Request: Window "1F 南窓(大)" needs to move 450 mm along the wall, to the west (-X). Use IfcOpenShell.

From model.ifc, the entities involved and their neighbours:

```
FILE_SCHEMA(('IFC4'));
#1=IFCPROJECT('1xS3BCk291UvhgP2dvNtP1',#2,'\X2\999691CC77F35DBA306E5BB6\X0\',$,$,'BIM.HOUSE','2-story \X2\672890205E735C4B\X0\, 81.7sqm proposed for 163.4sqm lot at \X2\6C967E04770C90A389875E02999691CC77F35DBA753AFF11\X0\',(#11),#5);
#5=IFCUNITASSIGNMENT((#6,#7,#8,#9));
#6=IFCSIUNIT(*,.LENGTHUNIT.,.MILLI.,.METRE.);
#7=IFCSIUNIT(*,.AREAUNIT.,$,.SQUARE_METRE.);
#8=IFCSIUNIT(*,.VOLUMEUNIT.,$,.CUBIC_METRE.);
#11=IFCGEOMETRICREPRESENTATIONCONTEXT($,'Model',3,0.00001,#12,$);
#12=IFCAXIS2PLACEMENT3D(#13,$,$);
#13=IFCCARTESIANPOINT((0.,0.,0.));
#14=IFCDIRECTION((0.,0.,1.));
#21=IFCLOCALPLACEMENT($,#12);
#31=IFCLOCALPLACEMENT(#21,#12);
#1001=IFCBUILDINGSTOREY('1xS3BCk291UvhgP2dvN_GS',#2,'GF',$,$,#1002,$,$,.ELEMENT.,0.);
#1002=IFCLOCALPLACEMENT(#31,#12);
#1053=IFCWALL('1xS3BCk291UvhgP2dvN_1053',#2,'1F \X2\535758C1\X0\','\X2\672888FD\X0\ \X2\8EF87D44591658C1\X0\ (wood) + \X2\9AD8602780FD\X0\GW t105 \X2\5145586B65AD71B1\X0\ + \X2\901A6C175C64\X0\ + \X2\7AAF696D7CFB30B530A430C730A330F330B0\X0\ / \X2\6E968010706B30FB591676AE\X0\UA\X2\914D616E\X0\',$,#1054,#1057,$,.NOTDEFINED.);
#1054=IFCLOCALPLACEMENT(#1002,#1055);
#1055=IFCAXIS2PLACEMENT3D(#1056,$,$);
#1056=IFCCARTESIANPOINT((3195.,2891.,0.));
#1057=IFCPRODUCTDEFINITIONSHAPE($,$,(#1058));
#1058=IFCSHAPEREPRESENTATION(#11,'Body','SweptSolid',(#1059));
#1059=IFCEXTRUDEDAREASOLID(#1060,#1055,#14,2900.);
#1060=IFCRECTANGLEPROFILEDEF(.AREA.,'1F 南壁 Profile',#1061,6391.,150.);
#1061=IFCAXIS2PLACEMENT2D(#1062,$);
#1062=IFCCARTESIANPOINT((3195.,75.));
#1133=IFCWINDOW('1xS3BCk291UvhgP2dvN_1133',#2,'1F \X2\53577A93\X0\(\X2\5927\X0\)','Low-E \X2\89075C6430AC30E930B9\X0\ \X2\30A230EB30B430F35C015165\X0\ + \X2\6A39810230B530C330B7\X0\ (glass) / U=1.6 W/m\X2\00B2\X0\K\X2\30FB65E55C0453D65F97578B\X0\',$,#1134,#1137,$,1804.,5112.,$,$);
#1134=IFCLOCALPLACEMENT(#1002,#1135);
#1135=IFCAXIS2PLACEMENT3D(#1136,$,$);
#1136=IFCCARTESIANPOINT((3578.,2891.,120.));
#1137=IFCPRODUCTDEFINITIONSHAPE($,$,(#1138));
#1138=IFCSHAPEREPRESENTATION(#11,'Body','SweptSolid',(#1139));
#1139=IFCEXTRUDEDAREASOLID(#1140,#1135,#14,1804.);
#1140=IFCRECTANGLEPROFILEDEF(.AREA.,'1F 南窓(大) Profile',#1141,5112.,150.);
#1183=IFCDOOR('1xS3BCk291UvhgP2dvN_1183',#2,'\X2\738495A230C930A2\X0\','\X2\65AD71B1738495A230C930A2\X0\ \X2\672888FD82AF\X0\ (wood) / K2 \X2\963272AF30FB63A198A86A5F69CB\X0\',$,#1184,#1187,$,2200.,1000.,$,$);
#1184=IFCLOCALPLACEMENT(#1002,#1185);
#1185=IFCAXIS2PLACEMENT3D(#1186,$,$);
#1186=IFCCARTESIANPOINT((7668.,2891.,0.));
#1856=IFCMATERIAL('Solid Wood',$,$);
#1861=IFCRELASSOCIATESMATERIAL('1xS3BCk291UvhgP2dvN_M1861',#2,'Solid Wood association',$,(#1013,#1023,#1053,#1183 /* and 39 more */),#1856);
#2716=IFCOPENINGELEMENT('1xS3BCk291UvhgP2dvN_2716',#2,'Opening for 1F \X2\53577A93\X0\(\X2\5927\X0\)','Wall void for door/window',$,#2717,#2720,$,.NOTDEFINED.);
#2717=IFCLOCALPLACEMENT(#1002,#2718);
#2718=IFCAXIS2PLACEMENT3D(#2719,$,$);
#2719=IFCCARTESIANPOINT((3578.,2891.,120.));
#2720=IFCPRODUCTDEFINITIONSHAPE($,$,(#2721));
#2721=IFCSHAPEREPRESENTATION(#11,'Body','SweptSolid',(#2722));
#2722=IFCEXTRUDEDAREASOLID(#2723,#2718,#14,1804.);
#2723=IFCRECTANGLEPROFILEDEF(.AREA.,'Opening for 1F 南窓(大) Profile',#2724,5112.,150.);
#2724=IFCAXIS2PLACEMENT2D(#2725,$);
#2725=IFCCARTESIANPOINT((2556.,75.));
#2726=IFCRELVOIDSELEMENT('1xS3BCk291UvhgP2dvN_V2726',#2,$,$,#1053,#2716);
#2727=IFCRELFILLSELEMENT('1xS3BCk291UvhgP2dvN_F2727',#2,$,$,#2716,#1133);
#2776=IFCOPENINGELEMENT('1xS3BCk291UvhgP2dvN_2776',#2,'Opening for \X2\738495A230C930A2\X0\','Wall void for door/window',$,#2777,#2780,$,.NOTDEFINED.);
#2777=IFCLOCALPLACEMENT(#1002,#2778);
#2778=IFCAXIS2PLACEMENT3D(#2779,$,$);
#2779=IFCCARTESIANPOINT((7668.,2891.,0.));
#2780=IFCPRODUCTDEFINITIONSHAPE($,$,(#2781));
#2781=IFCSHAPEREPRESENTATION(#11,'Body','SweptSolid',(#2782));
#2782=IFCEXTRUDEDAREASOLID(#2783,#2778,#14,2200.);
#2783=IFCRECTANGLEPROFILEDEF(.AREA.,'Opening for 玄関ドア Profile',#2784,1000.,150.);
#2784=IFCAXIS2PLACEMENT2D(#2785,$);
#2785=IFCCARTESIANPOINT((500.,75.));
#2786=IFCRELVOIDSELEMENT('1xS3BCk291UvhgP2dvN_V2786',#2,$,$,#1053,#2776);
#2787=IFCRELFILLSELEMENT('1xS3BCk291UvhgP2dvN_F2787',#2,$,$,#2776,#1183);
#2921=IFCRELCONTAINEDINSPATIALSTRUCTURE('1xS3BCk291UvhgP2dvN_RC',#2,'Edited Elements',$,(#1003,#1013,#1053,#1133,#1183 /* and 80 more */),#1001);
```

```python
import ifcopenshell
import ifcopenshell.api.geometry
import ifcopenshell.util.placement

model = ifcopenshell.open("model.ifc")

window = model.by_id(1133)
opening = window.FillsVoids[0].RelatingOpeningElement
wall = opening.VoidsElements[0].RelatingBuildingElement

wall_matrix = ifcopenshell.util.placement.get_local_placement(wall.ObjectPlacement)
shift = wall_matrix[:3, 0] * -450.0
before = ifcopenshell.util.placement.get_local_placement(window.ObjectPlacement)[:3, 3].copy()

# The window is not placed relative to its opening, so move both.
for product in (opening, window):
    matrix = ifcopenshell.util.placement.get_local_placement(product.ObjectPlacement)
    matrix[:3, 3] += shift
    ifcopenshell.api.geometry.edit_object_placement(model, product=product, matrix=matrix, is_si=False)

after = ifcopenshell.util.placement.get_local_placement(window.ObjectPlacement)[:3, 3]
print("window moved by", (after - before).round(3) + 0.0)

model.write("model_v2.ifc")
```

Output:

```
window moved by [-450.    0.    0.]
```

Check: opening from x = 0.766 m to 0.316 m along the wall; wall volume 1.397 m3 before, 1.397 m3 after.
